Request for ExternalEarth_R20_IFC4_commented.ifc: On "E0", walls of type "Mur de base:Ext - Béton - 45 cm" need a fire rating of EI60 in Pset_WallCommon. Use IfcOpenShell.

First a look at what the model holds.

```python
import ifcopenshell
import ifcopenshell.util.element

model = ifcopenshell.open("ExternalEarth_R20_IFC4_commented.ifc")
print(model.schema)
storey = next(s for s in model.by_type("IfcBuildingStorey") if s.Name == "E0")
walls = [e for e in ifcopenshell.util.element.get_decomposition(storey) if e.is_a("IfcWall")]
seen = {}
for e in walls:
    element_type = ifcopenshell.util.element.get_type(e)
    key = (element_type.Name if element_type != e and element_type else None, ifcopenshell.util.element.get_pset(e, "Pset_WallCommon", "FireRating"))
    seen[key] = seen.get(key, 0) + 1
for (name, value), count in sorted(seen.items(), key=str):
    print(count, "x", name, "|", value)
```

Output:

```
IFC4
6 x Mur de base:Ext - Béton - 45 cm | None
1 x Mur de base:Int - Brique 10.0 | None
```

```python
import ifcopenshell
import ifcopenshell.api.pset
import ifcopenshell.util.element

model = ifcopenshell.open("ExternalEarth_R20_IFC4_commented.ifc")

storey = next(s for s in model.by_type("IfcBuildingStorey") if s.Name == "E0")
walls = [e for e in ifcopenshell.util.element.get_decomposition(storey) if e.is_a("IfcWall")]

count = 0
for e in walls:
    element_type = ifcopenshell.util.element.get_type(e)
    if element_type in (None, e) or element_type.Name != "Mur de base:Ext - Béton - 45 cm":
        continue
    # add_pset returns the element's existing set when there is one.
    pset = ifcopenshell.api.pset.add_pset(model, product=e, name="Pset_WallCommon")
    ifcopenshell.api.pset.edit_pset(model, pset=pset, properties={"FireRating": "EI60"})
    count += 1

print(count, "walls updated")

model.write("ExternalEarth_R20_IFC4_commented_edited.ifc")
```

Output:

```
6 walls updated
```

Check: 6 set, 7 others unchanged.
